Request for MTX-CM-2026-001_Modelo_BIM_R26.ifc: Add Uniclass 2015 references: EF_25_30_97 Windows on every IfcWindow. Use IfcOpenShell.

First a look at what the model holds.

```python
import ifcopenshell

model = ifcopenshell.open("MTX-CM-2026-001_Modelo_BIM_R26.ifc")
print(model.schema)
print("classifications:", [c.Name for c in model.by_type("IfcClassification")])
for ifc_class in ("IfcDoor", "IfcRoof", "IfcStair", "IfcWall", "IfcWindow"):
    print(ifc_class, len(model.by_type(ifc_class)))
```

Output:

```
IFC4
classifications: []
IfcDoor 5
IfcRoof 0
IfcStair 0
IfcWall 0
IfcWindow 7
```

```python
import ifcopenshell
import ifcopenshell.api.classification

model = ifcopenshell.open("MTX-CM-2026-001_Modelo_BIM_R26.ifc")

system = ifcopenshell.api.classification.add_classification(model, classification="Uniclass 2015")

codes = {
    "IfcWindow": ("EF_25_30_97", "Windows"),
}
for ifc_class, (code, name) in codes.items():
    products = model.by_type(ifc_class)
    ifcopenshell.api.classification.add_reference(
        model, products=products, classification=system, identification=code, name=name
    )
    print(code, len(products))

model.write("MTX-CM-2026-001_Modelo_BIM_R26_v2.ifc")
```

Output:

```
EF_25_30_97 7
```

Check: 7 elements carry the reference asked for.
